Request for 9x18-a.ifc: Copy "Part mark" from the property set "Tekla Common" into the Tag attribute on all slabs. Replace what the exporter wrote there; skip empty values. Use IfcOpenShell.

First a look at what the model holds.

```python
import ifcopenshell
import ifcopenshell.util.element

model = ifcopenshell.open("9x18-a.ifc")
print(model.schema)
slabs = model.by_type("IfcSlab")
print(len(slabs), "slabs")
for e in slabs[:8]:
    source = ifcopenshell.util.element.get_pset(e, "Tekla Common", "Part mark")
    target = e.Tag
    print(e.id(), repr(source), repr(target), sep=" | ")
```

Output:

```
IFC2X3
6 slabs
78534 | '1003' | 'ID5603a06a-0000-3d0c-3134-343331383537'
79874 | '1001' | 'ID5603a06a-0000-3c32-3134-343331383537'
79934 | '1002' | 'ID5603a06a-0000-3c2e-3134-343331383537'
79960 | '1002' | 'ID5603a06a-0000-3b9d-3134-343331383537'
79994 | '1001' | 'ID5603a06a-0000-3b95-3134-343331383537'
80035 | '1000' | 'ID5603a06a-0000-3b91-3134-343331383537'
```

```python
import ifcopenshell
import ifcopenshell.util.element

model = ifcopenshell.open("9x18-a.ifc")

count = 0
for e in model.by_type("IfcSlab"):
    value = ifcopenshell.util.element.get_pset(e, "Tekla Common", "Part mark")
    current = e.Tag
    if not value or not value.strip() or current == value:
        continue
    e.Tag = value
    count += 1

print(count, "slabs updated")

model.write("9x18-a_edited.ifc")
```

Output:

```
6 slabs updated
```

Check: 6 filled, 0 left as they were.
